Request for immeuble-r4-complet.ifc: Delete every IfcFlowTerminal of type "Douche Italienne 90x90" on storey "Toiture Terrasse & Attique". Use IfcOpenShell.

First a look at what the model holds.

```python
import ifcopenshell
import ifcopenshell.util.element

model = ifcopenshell.open("immeuble-r4-complet.ifc")
print(model.schema)
storey = next(s for s in model.by_type("IfcBuildingStorey") if s.Name == "Toiture Terrasse & Attique")
terminals = [e for e in ifcopenshell.util.element.get_decomposition(storey) if e.is_a("IfcFlowTerminal")]
seen = {}
for e in terminals:
    element_type = ifcopenshell.util.element.get_type(e)
    name = element_type.Name if element_type not in (None, e) else None
    seen[name] = seen.get(name, 0) + 1
for name, count in sorted(seen.items(), key=str):
    print(count, "x", name)
```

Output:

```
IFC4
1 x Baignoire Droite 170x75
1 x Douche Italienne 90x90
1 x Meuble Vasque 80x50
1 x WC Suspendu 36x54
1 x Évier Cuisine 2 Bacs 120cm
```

```python
import ifcopenshell
import ifcopenshell.api.root
import ifcopenshell.util.element

model = ifcopenshell.open("immeuble-r4-complet.ifc")

storey = next(s for s in model.by_type("IfcBuildingStorey") if s.Name == "Toiture Terrasse & Attique")
terminals = [e for e in ifcopenshell.util.element.get_decomposition(storey) if e.is_a("IfcFlowTerminal")]
targets = [e for e in terminals if (t := ifcopenshell.util.element.get_type(e)) not in (None, e) and t.Name == "Douche Italienne 90x90"]

for e in targets:
    ifcopenshell.api.root.remove_product(model, product=e)
print(len(targets), "removed")

model.write("immeuble-r4-complet_updated.ifc")
```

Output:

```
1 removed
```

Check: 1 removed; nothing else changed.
